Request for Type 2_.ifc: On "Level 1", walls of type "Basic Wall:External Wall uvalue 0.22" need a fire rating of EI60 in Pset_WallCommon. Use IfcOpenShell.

First a look at what the model holds.

```python
import ifcopenshell
import ifcopenshell.util.element

model = ifcopenshell.open("Type 2_.ifc")
print(model.schema)
storey = next(s for s in model.by_type("IfcBuildingStorey") if s.Name == "Level 1")
walls = [e for e in ifcopenshell.util.element.get_decomposition(storey) if e.is_a("IfcWall")]
seen = {}
for e in walls:
    element_type = ifcopenshell.util.element.get_type(e)
    key = (element_type.Name if element_type != e and element_type else None, ifcopenshell.util.element.get_pset(e, "Pset_WallCommon", "FireRating"))
    seen[key] = seen.get(key, 0) + 1
for (name, value), count in sorted(seen.items(), key=str):
    print(count, "x", name, "|", value)
```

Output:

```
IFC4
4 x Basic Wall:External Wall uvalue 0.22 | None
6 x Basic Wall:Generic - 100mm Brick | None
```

```python
import ifcopenshell
import ifcopenshell.api.pset
import ifcopenshell.util.element

model = ifcopenshell.open("Type 2_.ifc")

storey = next(s for s in model.by_type("IfcBuildingStorey") if s.Name == "Level 1")
walls = [e for e in ifcopenshell.util.element.get_decomposition(storey) if e.is_a("IfcWall")]

count = 0
for e in walls:
    element_type = ifcopenshell.util.element.get_type(e)
    if element_type in (None, e) or element_type.Name != "Basic Wall:External Wall uvalue 0.22":
        continue
    # add_pset returns the element's existing set when there is one.
    pset = ifcopenshell.api.pset.add_pset(model, product=e, name="Pset_WallCommon")
    ifcopenshell.api.pset.edit_pset(model, pset=pset, properties={"FireRating": "EI60"})
    count += 1

print(count, "walls updated")

model.write("Type 2__edited.ifc")
```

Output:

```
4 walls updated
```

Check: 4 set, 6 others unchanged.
